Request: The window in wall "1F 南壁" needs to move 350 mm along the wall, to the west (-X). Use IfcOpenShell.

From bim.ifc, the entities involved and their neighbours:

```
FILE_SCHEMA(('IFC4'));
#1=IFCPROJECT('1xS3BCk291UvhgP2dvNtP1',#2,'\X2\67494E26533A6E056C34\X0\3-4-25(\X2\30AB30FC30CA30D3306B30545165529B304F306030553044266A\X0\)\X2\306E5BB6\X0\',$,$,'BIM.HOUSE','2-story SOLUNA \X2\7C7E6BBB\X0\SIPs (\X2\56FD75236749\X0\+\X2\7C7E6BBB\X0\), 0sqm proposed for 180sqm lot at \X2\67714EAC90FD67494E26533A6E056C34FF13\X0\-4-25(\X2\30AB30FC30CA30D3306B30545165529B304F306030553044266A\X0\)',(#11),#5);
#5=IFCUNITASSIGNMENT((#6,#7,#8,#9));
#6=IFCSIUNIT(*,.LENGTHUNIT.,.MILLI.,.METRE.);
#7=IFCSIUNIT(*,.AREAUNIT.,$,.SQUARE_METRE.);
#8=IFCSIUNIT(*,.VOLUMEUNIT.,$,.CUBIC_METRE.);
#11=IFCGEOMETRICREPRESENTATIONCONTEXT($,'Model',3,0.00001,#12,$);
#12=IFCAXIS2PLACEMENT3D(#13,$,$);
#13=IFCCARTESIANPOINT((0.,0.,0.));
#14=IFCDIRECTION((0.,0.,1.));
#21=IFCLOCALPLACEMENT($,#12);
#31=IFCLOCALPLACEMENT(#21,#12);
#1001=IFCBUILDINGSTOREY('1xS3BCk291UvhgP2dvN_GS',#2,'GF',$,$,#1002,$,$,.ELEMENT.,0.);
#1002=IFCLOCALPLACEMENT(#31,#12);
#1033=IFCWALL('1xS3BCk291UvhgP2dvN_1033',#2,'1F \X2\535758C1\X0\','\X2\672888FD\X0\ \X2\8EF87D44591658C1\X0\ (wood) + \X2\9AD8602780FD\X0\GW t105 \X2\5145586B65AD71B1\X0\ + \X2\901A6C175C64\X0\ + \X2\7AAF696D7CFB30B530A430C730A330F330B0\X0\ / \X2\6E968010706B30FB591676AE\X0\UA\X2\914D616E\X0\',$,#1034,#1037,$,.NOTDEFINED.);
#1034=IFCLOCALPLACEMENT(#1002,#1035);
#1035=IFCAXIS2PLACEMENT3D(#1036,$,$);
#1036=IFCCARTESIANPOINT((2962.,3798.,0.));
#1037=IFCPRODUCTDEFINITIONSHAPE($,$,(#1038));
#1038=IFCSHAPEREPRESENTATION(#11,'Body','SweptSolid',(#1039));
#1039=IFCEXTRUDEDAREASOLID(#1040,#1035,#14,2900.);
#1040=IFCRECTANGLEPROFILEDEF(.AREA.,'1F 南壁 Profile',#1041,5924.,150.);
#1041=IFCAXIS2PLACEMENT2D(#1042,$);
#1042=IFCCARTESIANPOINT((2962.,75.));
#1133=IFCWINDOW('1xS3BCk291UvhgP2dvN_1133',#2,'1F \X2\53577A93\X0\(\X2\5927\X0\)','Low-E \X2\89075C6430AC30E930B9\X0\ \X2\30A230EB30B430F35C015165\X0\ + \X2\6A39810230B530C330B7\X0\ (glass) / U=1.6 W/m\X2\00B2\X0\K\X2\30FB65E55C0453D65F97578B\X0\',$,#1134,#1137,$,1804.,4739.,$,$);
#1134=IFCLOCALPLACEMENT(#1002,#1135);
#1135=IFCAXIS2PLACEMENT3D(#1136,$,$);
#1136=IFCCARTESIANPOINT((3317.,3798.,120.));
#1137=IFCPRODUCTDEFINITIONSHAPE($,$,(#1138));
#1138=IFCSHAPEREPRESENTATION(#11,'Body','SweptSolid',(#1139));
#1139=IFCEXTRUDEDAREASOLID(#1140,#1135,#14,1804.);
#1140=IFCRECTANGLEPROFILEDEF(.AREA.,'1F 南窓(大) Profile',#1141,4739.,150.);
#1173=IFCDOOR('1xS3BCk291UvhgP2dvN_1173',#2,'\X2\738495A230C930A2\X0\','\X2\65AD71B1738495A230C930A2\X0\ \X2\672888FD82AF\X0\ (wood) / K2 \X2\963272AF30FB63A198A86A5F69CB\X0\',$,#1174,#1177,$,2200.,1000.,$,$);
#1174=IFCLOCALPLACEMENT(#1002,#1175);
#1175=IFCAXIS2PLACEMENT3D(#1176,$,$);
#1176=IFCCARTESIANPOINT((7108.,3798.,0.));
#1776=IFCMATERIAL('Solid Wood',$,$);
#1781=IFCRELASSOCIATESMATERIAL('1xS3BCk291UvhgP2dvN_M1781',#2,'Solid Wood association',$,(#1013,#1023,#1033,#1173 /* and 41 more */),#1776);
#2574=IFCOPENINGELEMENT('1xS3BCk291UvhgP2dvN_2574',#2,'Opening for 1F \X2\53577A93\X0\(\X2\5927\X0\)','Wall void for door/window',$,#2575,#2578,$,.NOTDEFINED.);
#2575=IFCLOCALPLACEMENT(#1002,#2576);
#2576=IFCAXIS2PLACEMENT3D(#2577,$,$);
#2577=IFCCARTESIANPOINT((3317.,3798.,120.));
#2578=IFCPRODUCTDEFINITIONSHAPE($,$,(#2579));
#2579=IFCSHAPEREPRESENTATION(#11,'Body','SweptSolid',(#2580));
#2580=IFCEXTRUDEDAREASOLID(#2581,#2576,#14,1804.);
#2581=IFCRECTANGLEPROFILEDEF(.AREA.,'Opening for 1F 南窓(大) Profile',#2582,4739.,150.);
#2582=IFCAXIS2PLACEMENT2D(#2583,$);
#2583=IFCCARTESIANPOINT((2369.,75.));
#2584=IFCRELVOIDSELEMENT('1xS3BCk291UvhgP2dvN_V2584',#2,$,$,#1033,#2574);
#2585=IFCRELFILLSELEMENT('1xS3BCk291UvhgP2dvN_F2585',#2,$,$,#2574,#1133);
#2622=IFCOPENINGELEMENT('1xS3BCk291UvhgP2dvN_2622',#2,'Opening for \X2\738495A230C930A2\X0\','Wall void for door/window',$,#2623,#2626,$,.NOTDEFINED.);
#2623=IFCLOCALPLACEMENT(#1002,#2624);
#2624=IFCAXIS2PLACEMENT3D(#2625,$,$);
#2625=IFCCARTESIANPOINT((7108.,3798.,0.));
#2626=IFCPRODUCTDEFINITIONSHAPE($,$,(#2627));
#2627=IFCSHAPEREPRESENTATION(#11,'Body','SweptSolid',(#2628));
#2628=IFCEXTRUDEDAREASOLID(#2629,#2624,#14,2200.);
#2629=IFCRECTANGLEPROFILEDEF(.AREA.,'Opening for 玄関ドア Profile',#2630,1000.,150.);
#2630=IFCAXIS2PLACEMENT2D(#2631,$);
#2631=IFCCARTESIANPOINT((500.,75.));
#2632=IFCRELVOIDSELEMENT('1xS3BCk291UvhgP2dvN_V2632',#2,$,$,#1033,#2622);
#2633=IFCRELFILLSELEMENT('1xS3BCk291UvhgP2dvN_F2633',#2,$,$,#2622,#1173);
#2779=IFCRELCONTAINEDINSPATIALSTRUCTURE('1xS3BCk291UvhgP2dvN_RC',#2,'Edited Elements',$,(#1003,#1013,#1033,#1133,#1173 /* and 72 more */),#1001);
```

```python
import ifcopenshell
import ifcopenshell.api.geometry
import ifcopenshell.util.placement

model = ifcopenshell.open("bim.ifc")

window = model.by_guid("1xS3BCk291UvhgP2dvN_1133")
opening = window.FillsVoids[0].RelatingOpeningElement
wall = opening.VoidsElements[0].RelatingBuildingElement

wall_matrix = ifcopenshell.util.placement.get_local_placement(wall.ObjectPlacement)
shift = wall_matrix[:3, 0] * -350.0
before = ifcopenshell.util.placement.get_local_placement(window.ObjectPlacement)[:3, 3].copy()

# The window is not placed relative to its opening, so move both.
for product in (opening, window):
    matrix = ifcopenshell.util.placement.get_local_placement(product.ObjectPlacement)
    matrix[:3, 3] += shift
    ifcopenshell.api.geometry.edit_object_placement(model, product=product, matrix=matrix, is_si=False)

after = ifcopenshell.util.placement.get_local_placement(window.ObjectPlacement)[:3, 3]
print("window moved by", (after - before).round(3) + 0.0)

model.write("bim_rev.ifc")
```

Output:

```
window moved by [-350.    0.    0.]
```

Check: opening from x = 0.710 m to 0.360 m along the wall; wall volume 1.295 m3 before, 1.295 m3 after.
